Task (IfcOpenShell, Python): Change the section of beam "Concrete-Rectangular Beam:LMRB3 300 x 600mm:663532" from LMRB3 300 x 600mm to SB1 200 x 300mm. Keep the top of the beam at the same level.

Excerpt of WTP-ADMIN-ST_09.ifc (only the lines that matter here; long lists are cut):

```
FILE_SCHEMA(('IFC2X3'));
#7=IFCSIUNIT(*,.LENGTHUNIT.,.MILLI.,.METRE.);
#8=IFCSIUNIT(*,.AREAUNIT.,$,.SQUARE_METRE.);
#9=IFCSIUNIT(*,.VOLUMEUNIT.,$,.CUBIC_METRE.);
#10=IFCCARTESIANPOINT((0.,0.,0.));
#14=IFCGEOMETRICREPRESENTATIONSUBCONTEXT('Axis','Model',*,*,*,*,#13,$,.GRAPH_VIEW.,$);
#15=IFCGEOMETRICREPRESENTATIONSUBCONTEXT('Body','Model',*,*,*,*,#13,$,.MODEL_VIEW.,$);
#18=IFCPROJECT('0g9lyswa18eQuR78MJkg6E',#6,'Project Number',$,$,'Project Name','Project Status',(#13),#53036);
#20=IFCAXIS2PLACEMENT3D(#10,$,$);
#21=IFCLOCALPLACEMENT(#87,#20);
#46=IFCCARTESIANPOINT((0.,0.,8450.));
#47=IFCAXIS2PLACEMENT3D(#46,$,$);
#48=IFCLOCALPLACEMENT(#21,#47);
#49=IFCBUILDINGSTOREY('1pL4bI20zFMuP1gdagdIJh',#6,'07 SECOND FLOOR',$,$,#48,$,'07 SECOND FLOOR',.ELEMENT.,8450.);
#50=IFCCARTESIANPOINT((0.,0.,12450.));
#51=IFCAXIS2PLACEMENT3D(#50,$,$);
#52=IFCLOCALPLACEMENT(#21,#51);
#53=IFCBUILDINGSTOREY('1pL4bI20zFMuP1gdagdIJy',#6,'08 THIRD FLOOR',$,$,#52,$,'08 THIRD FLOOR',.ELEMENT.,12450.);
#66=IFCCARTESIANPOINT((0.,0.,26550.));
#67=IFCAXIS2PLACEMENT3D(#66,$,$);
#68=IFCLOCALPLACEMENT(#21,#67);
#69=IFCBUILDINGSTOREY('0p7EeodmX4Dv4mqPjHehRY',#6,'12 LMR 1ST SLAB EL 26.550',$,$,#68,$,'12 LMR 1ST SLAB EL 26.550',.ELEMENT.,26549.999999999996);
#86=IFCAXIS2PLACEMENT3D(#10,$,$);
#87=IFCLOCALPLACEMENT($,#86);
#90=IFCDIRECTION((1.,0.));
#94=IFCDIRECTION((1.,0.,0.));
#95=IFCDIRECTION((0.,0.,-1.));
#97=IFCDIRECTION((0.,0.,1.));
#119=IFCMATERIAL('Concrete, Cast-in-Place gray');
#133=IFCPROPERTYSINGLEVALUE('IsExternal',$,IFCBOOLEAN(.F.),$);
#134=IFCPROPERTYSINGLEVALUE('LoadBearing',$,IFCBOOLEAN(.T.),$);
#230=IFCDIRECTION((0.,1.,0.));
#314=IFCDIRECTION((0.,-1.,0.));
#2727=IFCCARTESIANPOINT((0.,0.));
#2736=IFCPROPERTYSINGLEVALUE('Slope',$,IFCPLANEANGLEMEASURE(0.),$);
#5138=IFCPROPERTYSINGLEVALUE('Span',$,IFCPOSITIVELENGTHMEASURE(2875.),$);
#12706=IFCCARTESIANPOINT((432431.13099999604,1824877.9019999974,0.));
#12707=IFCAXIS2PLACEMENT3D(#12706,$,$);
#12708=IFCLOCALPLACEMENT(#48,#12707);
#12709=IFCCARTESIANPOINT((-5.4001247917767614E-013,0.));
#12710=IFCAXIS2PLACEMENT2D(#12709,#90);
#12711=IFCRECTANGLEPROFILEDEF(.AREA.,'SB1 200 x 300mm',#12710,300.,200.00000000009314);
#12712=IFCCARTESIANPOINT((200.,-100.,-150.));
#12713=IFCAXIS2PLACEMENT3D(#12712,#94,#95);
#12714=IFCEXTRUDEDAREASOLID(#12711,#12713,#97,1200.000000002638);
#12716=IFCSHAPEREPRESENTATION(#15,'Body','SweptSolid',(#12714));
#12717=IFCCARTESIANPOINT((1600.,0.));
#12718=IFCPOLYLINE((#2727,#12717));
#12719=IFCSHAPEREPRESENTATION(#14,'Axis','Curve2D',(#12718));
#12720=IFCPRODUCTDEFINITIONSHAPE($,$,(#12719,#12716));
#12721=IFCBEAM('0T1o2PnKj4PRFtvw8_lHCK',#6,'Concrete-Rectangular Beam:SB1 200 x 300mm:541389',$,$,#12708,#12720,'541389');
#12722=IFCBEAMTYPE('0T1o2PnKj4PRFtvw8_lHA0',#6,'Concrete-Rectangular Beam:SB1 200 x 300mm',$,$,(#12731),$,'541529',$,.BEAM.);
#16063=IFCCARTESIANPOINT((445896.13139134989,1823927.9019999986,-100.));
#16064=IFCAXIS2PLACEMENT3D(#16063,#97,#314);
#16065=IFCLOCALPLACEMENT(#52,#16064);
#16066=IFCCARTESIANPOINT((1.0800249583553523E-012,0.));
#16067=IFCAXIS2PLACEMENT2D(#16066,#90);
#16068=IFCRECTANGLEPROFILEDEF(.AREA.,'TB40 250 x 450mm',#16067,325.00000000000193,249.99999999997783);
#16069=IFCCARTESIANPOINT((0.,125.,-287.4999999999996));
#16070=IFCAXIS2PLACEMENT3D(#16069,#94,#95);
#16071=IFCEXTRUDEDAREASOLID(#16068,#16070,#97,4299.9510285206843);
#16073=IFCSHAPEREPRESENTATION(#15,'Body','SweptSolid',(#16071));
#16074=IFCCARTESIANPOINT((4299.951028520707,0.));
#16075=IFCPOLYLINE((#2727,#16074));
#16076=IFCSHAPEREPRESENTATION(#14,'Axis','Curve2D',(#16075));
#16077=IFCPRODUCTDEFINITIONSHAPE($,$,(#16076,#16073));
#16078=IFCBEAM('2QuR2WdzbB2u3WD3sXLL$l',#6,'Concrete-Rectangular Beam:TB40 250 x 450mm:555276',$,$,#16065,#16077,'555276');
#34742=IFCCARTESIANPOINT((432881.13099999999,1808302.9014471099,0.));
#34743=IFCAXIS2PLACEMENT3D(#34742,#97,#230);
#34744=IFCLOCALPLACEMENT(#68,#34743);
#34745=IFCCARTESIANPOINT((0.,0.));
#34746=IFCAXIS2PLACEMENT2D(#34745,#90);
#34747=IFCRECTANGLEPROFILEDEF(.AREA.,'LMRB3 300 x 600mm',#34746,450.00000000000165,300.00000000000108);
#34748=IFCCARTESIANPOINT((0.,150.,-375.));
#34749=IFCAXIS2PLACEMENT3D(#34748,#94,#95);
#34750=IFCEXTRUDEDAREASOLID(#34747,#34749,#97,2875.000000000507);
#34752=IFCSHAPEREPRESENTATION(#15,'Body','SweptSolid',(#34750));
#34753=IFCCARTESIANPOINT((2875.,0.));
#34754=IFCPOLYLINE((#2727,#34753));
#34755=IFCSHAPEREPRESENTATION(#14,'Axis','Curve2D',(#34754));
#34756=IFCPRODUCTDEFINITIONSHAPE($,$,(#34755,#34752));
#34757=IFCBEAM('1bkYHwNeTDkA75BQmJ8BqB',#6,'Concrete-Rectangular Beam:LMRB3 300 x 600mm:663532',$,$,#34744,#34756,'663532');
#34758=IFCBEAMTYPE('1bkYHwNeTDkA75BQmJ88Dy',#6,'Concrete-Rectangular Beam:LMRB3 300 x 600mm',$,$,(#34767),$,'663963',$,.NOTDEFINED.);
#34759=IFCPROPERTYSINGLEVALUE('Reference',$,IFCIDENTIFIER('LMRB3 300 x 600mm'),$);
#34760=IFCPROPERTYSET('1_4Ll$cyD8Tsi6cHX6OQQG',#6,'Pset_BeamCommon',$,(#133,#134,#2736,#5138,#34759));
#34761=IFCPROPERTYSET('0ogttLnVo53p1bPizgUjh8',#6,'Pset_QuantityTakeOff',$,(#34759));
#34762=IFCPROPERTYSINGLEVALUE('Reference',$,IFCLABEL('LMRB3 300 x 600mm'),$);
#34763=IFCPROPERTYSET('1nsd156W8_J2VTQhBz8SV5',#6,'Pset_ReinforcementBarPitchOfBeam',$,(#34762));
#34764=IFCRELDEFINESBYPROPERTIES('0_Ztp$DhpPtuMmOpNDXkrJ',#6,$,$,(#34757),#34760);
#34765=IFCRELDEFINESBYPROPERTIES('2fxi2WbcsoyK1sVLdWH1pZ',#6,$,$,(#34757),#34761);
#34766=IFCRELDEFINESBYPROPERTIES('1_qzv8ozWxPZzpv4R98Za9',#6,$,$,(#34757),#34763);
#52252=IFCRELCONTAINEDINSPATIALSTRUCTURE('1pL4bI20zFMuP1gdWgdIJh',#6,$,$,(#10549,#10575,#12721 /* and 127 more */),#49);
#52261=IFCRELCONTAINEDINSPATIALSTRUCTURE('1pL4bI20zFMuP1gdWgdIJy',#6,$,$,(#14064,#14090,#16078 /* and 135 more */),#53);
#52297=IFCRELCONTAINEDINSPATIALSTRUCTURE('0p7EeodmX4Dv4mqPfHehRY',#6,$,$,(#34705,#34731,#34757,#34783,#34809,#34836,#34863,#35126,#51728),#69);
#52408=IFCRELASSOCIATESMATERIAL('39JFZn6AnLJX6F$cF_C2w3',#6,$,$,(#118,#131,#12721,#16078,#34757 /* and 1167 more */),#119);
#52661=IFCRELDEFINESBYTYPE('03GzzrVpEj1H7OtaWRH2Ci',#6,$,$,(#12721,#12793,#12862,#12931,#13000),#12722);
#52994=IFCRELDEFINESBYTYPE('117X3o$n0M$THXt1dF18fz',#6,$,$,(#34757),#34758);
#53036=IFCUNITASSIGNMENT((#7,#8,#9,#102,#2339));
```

```python
import ifcopenshell
import ifcopenshell.api.pset
import ifcopenshell.api.type
import ifcopenshell.util.element
import ifcopenshell.util.representation

model = ifcopenshell.open("WTP-ADMIN-ST_09.ifc")

member = model.by_guid("1bkYHwNeTDkA75BQmJ8BqB")
source = next(p for p in model.by_type("IfcRectangleProfileDef") if p.ProfileName == "SB1 200 x 300mm")

body = ifcopenshell.util.representation.get_representation(member, "Model", "Body")
solid = body.Items[0]
old_profile = solid.SweptArea

# Copy the section's sizes but keep this member's own profile position.
profile = ifcopenshell.util.element.copy(model, source)
# Profiles are centred, so shift by half the change in depth to hold the top.
shift = (old_profile.XDim - profile.XDim) / 2
x, y = old_profile.Position.Location.Coordinates
up = (-1.0, 0.0)  # upwards, in the solid's own plane
location = model.createIfcCartesianPoint((x + up[0] * shift, y + up[1] * shift))
profile.Position = model.createIfcAxis2Placement2D(location, old_profile.Position.RefDirection)
solid.SweptArea = profile
if not model.get_total_inverses(old_profile):
    ifcopenshell.util.element.remove_deep2(model, old_profile)

new_type = model.by_guid("0T1o2PnKj4PRFtvw8_lHA0")
ifcopenshell.api.type.assign_type(
    model, related_objects=[member], relating_type=new_type, should_map_representations=False
)
member.Name = member.Name.replace("LMRB3 300 x 600mm", "SB1 200 x 300mm")
pset = model.by_id(ifcopenshell.util.element.get_pset(member, "Pset_BeamCommon", should_inherit=False)["id"])
ifcopenshell.api.pset.edit_pset(model, pset=pset, properties={"Reference": "SB1 200 x 300mm"})
pset = model.by_id(ifcopenshell.util.element.get_pset(member, "Pset_QuantityTakeOff", should_inherit=False)["id"])
ifcopenshell.api.pset.edit_pset(model, pset=pset, properties={"Reference": "SB1 200 x 300mm"})
pset = model.by_id(ifcopenshell.util.element.get_pset(member, "Pset_ReinforcementBarPitchOfBeam", should_inherit=False)["id"])
ifcopenshell.api.pset.edit_pset(model, pset=pset, properties={"Reference": "SB1 200 x 300mm"})

print(solid.SweptArea)

model.write("WTP-ADMIN-ST_09-out.ifc")
```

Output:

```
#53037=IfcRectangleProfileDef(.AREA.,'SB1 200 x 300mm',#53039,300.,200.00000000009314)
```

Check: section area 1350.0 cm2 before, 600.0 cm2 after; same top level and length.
